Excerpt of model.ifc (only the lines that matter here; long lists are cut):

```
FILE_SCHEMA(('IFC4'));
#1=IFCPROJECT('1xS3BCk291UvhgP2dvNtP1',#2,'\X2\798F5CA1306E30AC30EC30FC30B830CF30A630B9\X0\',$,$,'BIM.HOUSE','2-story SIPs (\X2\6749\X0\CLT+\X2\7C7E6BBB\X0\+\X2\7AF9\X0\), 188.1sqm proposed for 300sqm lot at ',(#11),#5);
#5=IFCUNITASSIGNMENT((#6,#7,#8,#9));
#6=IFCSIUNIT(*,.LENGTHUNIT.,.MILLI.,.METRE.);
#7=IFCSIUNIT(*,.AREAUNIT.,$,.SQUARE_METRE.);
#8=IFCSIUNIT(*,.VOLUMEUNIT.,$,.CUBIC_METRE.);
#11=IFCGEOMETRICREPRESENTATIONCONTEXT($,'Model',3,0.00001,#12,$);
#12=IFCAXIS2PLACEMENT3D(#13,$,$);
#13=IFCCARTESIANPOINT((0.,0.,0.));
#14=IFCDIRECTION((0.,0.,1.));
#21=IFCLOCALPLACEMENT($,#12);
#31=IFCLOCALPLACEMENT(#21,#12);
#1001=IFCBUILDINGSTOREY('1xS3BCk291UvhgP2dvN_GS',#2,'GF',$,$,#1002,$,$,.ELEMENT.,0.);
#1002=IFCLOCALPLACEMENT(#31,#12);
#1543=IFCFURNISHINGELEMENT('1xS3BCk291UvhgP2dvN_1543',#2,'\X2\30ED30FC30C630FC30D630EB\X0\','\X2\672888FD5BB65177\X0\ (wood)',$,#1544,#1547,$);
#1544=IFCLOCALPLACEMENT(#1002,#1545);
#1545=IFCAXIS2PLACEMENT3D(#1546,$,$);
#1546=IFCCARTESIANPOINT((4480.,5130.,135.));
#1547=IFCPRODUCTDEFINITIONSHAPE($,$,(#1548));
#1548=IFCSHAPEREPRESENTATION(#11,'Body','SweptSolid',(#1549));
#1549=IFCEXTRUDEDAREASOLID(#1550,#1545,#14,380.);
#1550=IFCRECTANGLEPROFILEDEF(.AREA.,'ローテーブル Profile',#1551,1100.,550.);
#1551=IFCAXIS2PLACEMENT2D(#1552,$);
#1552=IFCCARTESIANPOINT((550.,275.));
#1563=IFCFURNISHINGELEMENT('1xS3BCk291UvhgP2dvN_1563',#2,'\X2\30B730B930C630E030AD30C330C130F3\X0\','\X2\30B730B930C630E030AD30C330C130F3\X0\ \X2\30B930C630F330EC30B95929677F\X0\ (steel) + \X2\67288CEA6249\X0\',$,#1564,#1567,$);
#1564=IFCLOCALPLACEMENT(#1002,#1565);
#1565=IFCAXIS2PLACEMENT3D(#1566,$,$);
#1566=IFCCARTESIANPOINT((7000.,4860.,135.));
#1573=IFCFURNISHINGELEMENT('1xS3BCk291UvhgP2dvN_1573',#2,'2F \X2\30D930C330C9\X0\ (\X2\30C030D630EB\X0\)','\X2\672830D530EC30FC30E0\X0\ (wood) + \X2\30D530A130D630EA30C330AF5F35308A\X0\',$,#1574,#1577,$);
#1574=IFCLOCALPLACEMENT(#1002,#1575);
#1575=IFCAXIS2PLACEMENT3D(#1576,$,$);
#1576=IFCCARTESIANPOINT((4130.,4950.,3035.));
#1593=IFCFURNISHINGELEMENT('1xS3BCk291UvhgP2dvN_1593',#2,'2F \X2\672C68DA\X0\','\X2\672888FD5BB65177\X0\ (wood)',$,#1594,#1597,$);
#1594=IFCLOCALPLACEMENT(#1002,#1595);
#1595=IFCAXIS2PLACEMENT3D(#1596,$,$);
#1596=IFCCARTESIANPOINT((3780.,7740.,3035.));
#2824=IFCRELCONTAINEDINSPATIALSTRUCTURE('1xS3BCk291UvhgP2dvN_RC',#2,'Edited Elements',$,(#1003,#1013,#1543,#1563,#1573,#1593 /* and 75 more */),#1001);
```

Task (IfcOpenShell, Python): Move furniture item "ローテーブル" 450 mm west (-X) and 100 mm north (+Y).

```python
import ifcopenshell
import ifcopenshell.api.geometry
import ifcopenshell.util.placement
import ifcopenshell.util.unit

model = ifcopenshell.open("model.ifc")
unit_scale = ifcopenshell.util.unit.calculate_unit_scale(model)

item = model.by_guid("1xS3BCk291UvhgP2dvN_1543")
matrix = ifcopenshell.util.placement.get_local_placement(item.ObjectPlacement)
matrix[0, 3] -= 0.45 / unit_scale
matrix[1, 3] += 0.1 / unit_scale
ifcopenshell.api.geometry.edit_object_placement(model, product=item, matrix=matrix, is_si=False)

print(ifcopenshell.util.placement.get_local_placement(item.ObjectPlacement).round(3) + 0.0)

model.write("model_rev.ifc")
```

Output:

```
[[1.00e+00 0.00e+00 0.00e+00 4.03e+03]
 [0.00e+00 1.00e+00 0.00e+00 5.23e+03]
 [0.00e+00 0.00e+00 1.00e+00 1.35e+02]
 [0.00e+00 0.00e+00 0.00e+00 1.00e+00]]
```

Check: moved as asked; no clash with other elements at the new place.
